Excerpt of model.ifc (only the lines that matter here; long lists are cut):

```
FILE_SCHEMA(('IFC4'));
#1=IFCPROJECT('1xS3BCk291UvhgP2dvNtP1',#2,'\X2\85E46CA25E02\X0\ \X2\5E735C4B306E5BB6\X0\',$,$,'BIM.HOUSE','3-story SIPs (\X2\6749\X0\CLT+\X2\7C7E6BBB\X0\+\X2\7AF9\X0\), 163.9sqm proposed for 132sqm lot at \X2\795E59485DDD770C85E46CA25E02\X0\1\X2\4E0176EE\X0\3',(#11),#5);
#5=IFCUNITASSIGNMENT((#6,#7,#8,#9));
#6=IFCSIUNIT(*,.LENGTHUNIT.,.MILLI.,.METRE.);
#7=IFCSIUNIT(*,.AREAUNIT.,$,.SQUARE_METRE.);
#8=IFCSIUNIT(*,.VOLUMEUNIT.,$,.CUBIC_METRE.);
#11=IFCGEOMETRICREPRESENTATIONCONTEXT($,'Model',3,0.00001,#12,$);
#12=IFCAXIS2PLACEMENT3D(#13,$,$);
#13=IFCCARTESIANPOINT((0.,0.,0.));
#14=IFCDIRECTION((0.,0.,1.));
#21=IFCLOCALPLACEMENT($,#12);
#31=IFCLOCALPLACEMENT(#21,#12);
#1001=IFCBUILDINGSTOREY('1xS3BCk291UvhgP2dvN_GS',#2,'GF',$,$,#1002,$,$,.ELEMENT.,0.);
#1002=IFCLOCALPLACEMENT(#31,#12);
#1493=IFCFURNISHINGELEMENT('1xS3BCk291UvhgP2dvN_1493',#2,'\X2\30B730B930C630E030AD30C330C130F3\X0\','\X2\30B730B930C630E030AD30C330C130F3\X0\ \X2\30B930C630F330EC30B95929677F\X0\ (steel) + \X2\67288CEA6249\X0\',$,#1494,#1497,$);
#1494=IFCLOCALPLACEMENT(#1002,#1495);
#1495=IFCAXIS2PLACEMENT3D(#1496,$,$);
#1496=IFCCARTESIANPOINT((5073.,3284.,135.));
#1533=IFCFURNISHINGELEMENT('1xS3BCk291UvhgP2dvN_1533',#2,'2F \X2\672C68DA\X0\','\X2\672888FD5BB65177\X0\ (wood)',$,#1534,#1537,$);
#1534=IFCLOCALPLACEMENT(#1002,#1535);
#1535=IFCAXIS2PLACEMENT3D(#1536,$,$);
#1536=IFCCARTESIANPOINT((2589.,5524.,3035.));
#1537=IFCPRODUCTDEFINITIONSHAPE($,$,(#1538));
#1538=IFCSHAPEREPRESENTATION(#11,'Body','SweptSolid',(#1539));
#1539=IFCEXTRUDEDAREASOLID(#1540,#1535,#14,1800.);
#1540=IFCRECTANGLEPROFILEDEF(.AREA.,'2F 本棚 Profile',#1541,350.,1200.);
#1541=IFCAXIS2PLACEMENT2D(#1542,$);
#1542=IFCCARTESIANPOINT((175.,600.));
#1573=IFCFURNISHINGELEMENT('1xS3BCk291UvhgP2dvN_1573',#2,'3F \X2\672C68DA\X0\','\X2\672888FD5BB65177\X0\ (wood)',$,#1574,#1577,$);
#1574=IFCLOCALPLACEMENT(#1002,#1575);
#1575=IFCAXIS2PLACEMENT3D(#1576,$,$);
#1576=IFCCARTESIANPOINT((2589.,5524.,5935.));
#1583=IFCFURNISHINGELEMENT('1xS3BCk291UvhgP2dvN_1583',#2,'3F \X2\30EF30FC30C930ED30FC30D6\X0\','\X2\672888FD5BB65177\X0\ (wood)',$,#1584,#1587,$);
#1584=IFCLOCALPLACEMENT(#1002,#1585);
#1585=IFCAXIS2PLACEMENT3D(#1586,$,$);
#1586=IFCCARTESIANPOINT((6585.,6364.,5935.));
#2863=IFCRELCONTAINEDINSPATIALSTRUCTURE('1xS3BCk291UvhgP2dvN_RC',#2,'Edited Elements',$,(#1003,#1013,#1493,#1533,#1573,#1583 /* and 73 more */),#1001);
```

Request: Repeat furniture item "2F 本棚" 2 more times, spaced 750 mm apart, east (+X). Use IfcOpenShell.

```python
import numpy as np
import ifcopenshell
import ifcopenshell.api.geometry
import ifcopenshell.api.root
import ifcopenshell.util.element
import ifcopenshell.util.placement
import ifcopenshell.util.unit

model = ifcopenshell.open("model.ifc")
unit_scale = ifcopenshell.util.unit.calculate_unit_scale(model)


def reuse_history(source, copy):
    """copy_class also copies each property set's owner history, people and application; keep the originals."""
    for rel in copy.IsDefinedBy:
        if rel.is_a("IfcRelDefinesByProperties") and (history := rel.RelatingPropertyDefinition.OwnerHistory):
            rel.RelatingPropertyDefinition.OwnerHistory = source.OwnerHistory
            ifcopenshell.util.element.remove_deep2(model, history)


source = model.by_id(1533)
base = ifcopenshell.util.placement.get_local_placement(source.ObjectPlacement)
step = np.array([1.0, 0.0, 0.0]) * 0.75 / unit_scale

for i in range(1, 3):
    copy = ifcopenshell.api.root.copy_class(model, product=source)
    copy.Representation = ifcopenshell.util.element.copy_deep(
        model, source.Representation, exclude=["IfcGeometricRepresentationContext", "IfcRepresentationMap"]
    )
    reuse_history(source, copy)
    matrix = base.copy()
    matrix[:3, 3] += i * step
    print("added at", matrix[:3, 3].round(3) + 0.0)
    ifcopenshell.api.geometry.edit_object_placement(model, product=copy, matrix=matrix, is_si=False)

model.write("model_rev.ifc")
```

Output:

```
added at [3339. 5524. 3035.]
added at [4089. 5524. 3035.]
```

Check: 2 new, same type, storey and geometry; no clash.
